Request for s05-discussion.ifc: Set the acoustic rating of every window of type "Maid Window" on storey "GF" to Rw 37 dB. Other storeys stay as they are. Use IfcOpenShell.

First a look at what the model holds.

```python
import ifcopenshell
import ifcopenshell.util.element

model = ifcopenshell.open("s05-discussion.ifc")
print(model.schema)
storey = next(s for s in model.by_type("IfcBuildingStorey") if s.Name == "GF")
windows = [e for e in ifcopenshell.util.element.get_decomposition(storey) if e.is_a("IfcWindow")]
seen = {}
for e in windows:
    element_type = ifcopenshell.util.element.get_type(e)
    key = (element_type.Name if element_type != e and element_type else None, ifcopenshell.util.element.get_pset(e, "Pset_WindowCommon", "AcousticRating"))
    seen[key] = seen.get(key, 0) + 1
for (name, value), count in sorted(seen.items(), key=str):
    print(count, "x", name, "|", value)
```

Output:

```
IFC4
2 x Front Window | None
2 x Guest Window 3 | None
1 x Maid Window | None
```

```python
import ifcopenshell
import ifcopenshell.api.pset
import ifcopenshell.util.element

model = ifcopenshell.open("s05-discussion.ifc")

storey = next(s for s in model.by_type("IfcBuildingStorey") if s.Name == "GF")
windows = [e for e in ifcopenshell.util.element.get_decomposition(storey) if e.is_a("IfcWindow")]

count = 0
for e in windows:
    element_type = ifcopenshell.util.element.get_type(e)
    if element_type in (None, e) or element_type.Name != "Maid Window":
        continue
    # add_pset returns the element's existing set when there is one.
    pset = ifcopenshell.api.pset.add_pset(model, product=e, name="Pset_WindowCommon")
    ifcopenshell.api.pset.edit_pset(model, pset=pset, properties={"AcousticRating": "Rw 37 dB"})
    count += 1

print(count, "windows updated")

model.write("s05-discussion-out.ifc")
```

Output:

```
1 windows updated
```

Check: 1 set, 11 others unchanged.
